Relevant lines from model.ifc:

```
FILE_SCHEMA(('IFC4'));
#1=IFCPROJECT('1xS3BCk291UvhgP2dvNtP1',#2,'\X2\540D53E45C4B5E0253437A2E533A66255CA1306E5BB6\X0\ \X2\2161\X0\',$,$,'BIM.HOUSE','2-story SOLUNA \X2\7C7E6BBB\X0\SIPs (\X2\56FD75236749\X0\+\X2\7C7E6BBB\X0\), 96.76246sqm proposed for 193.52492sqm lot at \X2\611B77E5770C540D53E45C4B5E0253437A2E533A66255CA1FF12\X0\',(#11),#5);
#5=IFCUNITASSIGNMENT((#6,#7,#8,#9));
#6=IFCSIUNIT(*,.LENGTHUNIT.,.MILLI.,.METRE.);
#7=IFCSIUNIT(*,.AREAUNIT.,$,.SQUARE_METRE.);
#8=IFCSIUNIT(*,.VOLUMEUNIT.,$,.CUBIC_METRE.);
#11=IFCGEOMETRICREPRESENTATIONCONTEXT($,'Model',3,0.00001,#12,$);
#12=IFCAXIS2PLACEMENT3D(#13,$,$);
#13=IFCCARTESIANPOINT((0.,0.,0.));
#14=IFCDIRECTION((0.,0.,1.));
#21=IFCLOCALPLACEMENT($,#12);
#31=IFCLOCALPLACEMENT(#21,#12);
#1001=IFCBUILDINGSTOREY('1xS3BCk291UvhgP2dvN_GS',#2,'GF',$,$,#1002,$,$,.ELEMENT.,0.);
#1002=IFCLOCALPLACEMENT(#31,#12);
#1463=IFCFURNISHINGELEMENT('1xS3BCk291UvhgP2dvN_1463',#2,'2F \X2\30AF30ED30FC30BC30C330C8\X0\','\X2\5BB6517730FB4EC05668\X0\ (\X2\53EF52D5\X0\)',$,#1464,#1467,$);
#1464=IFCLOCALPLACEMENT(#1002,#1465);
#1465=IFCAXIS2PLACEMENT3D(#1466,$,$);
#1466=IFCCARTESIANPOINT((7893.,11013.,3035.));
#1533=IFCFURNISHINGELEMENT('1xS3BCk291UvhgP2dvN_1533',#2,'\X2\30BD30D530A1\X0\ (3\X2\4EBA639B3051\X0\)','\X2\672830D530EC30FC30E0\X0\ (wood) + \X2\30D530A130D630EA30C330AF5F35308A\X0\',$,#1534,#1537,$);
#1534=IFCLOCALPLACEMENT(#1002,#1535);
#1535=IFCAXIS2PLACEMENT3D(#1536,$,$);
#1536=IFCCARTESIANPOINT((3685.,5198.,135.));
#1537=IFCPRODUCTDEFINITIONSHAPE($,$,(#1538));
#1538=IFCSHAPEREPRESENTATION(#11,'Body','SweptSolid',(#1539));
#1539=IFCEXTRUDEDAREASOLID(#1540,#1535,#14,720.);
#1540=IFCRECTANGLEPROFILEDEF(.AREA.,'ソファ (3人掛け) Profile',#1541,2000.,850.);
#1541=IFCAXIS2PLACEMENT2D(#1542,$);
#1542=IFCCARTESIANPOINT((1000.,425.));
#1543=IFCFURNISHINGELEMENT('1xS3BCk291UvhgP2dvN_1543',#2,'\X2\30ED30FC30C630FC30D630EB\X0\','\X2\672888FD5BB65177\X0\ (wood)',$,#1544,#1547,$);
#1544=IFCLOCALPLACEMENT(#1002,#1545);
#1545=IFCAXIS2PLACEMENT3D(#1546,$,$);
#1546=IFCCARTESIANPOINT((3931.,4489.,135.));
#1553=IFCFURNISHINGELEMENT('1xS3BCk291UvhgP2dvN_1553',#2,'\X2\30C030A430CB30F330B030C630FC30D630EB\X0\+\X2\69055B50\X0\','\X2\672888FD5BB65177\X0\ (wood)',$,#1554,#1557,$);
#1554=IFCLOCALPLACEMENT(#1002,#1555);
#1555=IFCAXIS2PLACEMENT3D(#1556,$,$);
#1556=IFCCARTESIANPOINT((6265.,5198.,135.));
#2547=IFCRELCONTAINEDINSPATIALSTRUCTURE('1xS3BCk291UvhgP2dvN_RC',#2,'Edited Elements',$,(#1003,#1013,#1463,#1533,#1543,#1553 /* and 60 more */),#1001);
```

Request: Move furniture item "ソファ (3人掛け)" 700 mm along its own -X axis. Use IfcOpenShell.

```python
import ifcopenshell
import ifcopenshell.api.geometry
import ifcopenshell.util.placement
import ifcopenshell.util.unit

model = ifcopenshell.open("model.ifc")
unit_scale = ifcopenshell.util.unit.calculate_unit_scale(model)

item = model.by_guid("1xS3BCk291UvhgP2dvN_1533")
matrix = ifcopenshell.util.placement.get_local_placement(item.ObjectPlacement)
matrix[:3, 3] -= matrix[:3, 0] * 0.7 / unit_scale
ifcopenshell.api.geometry.edit_object_placement(model, product=item, matrix=matrix, is_si=False)

print(ifcopenshell.util.placement.get_local_placement(item.ObjectPlacement).round(3) + 0.0)

model.write("model-out.ifc")
```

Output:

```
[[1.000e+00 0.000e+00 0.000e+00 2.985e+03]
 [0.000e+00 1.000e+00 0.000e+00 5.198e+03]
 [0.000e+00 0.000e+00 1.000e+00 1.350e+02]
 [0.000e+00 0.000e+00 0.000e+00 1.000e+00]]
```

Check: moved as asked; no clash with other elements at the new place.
